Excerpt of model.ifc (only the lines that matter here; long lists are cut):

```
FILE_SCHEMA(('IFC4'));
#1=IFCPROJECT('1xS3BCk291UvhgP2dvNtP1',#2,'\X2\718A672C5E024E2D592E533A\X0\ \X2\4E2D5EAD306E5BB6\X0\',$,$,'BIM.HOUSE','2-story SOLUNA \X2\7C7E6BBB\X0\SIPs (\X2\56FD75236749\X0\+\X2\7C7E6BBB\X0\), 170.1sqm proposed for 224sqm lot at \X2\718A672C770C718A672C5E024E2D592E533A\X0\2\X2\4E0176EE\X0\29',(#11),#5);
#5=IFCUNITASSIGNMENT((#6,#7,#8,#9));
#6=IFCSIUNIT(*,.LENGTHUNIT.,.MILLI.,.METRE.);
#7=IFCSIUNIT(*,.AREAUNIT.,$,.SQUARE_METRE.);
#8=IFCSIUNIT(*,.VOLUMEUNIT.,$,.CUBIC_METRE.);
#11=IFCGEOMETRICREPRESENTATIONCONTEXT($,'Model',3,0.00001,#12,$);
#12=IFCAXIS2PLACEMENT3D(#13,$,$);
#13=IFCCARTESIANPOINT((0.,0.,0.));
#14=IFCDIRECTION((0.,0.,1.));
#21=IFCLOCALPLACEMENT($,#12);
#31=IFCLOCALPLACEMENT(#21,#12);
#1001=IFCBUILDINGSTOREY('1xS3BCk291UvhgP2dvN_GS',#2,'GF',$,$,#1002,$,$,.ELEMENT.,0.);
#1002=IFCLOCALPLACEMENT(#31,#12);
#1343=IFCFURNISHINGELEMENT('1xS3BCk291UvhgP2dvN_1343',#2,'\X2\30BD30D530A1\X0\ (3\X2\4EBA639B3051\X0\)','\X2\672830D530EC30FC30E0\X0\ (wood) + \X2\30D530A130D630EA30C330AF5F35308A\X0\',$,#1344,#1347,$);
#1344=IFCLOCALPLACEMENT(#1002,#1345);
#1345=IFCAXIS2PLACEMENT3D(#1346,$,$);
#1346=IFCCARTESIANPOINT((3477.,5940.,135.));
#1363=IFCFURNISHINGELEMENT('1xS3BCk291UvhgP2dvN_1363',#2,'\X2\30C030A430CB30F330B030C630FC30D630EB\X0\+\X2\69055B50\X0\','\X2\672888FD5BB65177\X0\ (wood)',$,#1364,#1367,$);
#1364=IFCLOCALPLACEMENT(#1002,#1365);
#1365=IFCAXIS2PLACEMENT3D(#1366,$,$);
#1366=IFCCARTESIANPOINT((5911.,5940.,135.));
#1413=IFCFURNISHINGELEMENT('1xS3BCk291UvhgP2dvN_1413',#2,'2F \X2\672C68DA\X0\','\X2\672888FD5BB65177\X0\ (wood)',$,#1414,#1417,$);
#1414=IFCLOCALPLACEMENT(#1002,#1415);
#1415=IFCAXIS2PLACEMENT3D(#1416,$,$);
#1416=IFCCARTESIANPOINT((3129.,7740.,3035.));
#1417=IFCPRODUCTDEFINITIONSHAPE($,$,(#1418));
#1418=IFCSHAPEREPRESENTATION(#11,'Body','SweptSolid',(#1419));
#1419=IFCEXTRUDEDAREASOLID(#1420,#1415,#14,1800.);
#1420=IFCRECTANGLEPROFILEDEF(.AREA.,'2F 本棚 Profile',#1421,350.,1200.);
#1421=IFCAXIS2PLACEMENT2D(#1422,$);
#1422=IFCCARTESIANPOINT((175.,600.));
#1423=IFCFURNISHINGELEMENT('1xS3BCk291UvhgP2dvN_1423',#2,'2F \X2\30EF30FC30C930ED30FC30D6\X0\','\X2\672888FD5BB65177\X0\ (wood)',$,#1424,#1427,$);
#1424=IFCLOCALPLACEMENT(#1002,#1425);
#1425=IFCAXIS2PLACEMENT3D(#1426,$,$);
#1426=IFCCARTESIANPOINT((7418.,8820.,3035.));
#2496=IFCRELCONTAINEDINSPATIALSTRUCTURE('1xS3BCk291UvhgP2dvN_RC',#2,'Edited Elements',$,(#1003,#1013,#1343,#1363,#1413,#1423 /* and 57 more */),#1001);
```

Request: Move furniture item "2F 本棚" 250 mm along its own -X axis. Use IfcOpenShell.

```python
import ifcopenshell
import ifcopenshell.api.geometry
import ifcopenshell.util.placement
import ifcopenshell.util.unit

model = ifcopenshell.open("model.ifc")
unit_scale = ifcopenshell.util.unit.calculate_unit_scale(model)

item = model.by_guid("1xS3BCk291UvhgP2dvN_1413")
matrix = ifcopenshell.util.placement.get_local_placement(item.ObjectPlacement)
matrix[:3, 3] -= matrix[:3, 0] * 0.25 / unit_scale
ifcopenshell.api.geometry.edit_object_placement(model, product=item, matrix=matrix, is_si=False)

print(ifcopenshell.util.placement.get_local_placement(item.ObjectPlacement).round(3) + 0.0)

model.write("model-out.ifc")
```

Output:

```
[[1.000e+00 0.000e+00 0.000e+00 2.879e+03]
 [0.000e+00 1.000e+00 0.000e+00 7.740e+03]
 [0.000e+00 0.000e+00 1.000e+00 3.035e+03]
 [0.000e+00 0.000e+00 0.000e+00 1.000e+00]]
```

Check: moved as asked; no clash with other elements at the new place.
